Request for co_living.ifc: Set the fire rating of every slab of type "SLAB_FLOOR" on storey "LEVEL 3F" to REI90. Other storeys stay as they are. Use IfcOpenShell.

First a look at what the model holds.

```python
import ifcopenshell
import ifcopenshell.util.element

model = ifcopenshell.open("co_living.ifc")
print(model.schema)
storey = next(s for s in model.by_type("IfcBuildingStorey") if s.Name == "LEVEL 3F")
slabs = [e for e in ifcopenshell.util.element.get_decomposition(storey) if e.is_a("IfcSlab")]
seen = {}
for e in slabs:
    element_type = ifcopenshell.util.element.get_type(e)
    key = (element_type.Name if element_type != e and element_type else None, ifcopenshell.util.element.get_pset(e, "Pset_SlabCommon", "FireRating"))
    seen[key] = seen.get(key, 0) + 1
for (name, value), count in sorted(seen.items(), key=str):
    print(count, "x", name, "|", value)
```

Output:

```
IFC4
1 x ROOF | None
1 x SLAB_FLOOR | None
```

```python
import ifcopenshell
import ifcopenshell.api.pset
import ifcopenshell.util.element

model = ifcopenshell.open("co_living.ifc")

storey = next(s for s in model.by_type("IfcBuildingStorey") if s.Name == "LEVEL 3F")
slabs = [e for e in ifcopenshell.util.element.get_decomposition(storey) if e.is_a("IfcSlab")]

count = 0
for e in slabs:
    element_type = ifcopenshell.util.element.get_type(e)
    if element_type in (None, e) or element_type.Name != "SLAB_FLOOR":
        continue
    # add_pset returns the element's existing set when there is one.
    pset = ifcopenshell.api.pset.add_pset(model, product=e, name="Pset_SlabCommon")
    ifcopenshell.api.pset.edit_pset(model, pset=pset, properties={"FireRating": "REI90"})
    count += 1

print(count, "slabs updated")

model.write("co_living-out.ifc")
```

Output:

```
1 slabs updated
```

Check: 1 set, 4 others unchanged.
